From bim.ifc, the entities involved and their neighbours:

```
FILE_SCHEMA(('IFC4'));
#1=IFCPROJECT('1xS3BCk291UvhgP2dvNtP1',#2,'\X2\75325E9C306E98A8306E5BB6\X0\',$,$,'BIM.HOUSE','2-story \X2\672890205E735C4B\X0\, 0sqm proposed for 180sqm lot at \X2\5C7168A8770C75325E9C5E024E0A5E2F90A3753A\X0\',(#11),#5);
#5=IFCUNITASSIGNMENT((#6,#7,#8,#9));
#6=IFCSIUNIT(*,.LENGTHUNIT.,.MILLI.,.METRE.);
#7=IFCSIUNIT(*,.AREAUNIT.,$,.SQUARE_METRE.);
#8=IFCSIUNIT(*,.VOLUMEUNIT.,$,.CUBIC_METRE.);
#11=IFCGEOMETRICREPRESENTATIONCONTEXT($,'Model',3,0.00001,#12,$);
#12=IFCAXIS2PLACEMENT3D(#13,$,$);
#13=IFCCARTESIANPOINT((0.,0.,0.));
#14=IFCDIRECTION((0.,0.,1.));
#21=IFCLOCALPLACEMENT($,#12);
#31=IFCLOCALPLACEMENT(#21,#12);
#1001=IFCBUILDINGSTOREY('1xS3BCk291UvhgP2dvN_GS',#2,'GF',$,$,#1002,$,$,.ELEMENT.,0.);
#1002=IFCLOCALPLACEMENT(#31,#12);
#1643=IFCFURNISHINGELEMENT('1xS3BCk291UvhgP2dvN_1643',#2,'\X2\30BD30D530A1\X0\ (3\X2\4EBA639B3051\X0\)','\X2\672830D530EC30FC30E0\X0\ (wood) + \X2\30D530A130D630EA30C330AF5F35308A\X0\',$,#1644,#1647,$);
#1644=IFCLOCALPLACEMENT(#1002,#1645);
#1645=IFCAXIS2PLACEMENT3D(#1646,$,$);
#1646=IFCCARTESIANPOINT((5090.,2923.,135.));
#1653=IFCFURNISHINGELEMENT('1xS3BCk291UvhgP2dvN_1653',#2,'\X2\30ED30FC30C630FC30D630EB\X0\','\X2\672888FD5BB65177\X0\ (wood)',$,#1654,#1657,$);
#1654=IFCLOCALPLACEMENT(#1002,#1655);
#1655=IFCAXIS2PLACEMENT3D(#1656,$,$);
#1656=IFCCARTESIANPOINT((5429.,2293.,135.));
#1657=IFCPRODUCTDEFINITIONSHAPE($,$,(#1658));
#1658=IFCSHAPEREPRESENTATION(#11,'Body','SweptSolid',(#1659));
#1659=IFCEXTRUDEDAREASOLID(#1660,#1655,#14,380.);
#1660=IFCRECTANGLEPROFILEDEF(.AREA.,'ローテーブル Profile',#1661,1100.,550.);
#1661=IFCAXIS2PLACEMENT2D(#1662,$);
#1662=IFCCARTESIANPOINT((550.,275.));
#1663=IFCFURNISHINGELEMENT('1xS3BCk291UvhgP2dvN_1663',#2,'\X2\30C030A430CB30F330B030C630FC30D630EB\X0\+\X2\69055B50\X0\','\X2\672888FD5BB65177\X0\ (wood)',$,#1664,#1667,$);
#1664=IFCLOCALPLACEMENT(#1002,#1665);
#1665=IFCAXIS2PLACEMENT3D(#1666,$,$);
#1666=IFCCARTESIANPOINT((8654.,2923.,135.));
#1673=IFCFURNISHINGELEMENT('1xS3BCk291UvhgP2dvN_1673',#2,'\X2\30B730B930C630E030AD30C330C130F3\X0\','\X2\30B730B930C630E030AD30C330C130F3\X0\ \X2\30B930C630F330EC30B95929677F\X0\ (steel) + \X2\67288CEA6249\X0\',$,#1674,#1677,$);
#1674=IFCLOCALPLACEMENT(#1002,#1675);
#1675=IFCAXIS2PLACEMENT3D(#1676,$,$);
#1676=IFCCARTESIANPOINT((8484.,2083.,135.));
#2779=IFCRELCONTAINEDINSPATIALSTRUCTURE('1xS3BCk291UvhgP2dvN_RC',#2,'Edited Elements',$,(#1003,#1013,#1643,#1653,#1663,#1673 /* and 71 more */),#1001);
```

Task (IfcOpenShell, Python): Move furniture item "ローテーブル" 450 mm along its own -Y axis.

```python
import ifcopenshell
import ifcopenshell.api.geometry
import ifcopenshell.util.placement
import ifcopenshell.util.unit

model = ifcopenshell.open("bim.ifc")
unit_scale = ifcopenshell.util.unit.calculate_unit_scale(model)

item = model.by_guid("1xS3BCk291UvhgP2dvN_1653")
matrix = ifcopenshell.util.placement.get_local_placement(item.ObjectPlacement)
matrix[:3, 3] -= matrix[:3, 1] * 0.45 / unit_scale
ifcopenshell.api.geometry.edit_object_placement(model, product=item, matrix=matrix, is_si=False)

print(ifcopenshell.util.placement.get_local_placement(item.ObjectPlacement).round(3) + 0.0)

model.write("bim_rev.ifc")
```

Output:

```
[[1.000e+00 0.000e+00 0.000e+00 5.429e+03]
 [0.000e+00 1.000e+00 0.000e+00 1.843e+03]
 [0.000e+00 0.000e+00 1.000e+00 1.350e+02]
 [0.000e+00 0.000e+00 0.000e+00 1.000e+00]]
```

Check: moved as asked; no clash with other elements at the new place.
